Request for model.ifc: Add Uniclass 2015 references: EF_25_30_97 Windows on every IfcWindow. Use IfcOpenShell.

First a look at what the model holds.

```python
import ifcopenshell

model = ifcopenshell.open("model.ifc")
print(model.schema)
print("classifications:", [c.Name for c in model.by_type("IfcClassification")])
for ifc_class in ("IfcDoor", "IfcRoof", "IfcStair", "IfcWall", "IfcWindow"):
    print(ifc_class, len(model.by_type(ifc_class)))
```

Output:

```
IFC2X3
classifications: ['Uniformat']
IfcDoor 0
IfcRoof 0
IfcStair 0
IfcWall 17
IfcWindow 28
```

```python
import ifcopenshell
import ifcopenshell.api.classification

model = ifcopenshell.open("model.ifc")

# IFC2X3 requires Source and Edition and has no link from the project to the system.
system = model.create_entity("IfcClassification", Source="NBS", Edition="2015", Name="Uniclass 2015")

codes = {
    "IfcWindow": ("EF_25_30_97", "Windows"),
}
for ifc_class, (code, name) in codes.items():
    products = model.by_type(ifc_class)
    ifcopenshell.api.classification.add_reference(
        model, products=products, classification=system, identification=code, name=name
    )
    print(code, len(products))

model.write("model_updated.ifc")
```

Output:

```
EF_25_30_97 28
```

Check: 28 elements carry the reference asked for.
